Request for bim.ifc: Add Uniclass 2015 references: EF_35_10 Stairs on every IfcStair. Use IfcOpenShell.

First a look at what the model holds.

```python
import ifcopenshell

model = ifcopenshell.open("bim.ifc")
print(model.schema)
print("classifications:", [c.Name for c in model.by_type("IfcClassification")])
for ifc_class in ("IfcDoor", "IfcRoof", "IfcStair", "IfcWall", "IfcWindow"):
    print(ifc_class, len(model.by_type(ifc_class)))
```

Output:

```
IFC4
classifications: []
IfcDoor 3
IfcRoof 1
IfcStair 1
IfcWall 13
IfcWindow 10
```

```python
import ifcopenshell
import ifcopenshell.api.classification

model = ifcopenshell.open("bim.ifc")

system = ifcopenshell.api.classification.add_classification(model, classification="Uniclass 2015")

codes = {
    "IfcStair": ("EF_35_10", "Stairs"),
}
for ifc_class, (code, name) in codes.items():
    products = model.by_type(ifc_class)
    ifcopenshell.api.classification.add_reference(
        model, products=products, classification=system, identification=code, name=name
    )
    print(code, len(products))

model.write("bim_v2.ifc")
```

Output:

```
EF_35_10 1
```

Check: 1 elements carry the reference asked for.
